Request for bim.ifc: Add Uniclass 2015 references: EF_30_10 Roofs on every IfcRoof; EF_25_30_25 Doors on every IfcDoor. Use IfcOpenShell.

First a look at what the model holds.

```python
import ifcopenshell

model = ifcopenshell.open("bim.ifc")
print(model.schema)
print("classifications:", [c.Name for c in model.by_type("IfcClassification")])
for ifc_class in ("IfcDoor", "IfcRoof", "IfcStair", "IfcWall", "IfcWindow"):
    print(ifc_class, len(model.by_type(ifc_class)))
```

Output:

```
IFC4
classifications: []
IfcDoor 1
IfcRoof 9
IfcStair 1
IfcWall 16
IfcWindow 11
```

```python
import ifcopenshell
import ifcopenshell.api.classification

model = ifcopenshell.open("bim.ifc")

system = ifcopenshell.api.classification.add_classification(model, classification="Uniclass 2015")

codes = {
    "IfcRoof": ("EF_30_10", "Roofs"),
    "IfcDoor": ("EF_25_30_25", "Doors"),
}
for ifc_class, (code, name) in codes.items():
    products = model.by_type(ifc_class)
    ifcopenshell.api.classification.add_reference(
        model, products=products, classification=system, identification=code, name=name
    )
    print(code, len(products))

model.write("bim-out.ifc")
```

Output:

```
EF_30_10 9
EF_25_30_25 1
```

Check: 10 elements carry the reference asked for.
